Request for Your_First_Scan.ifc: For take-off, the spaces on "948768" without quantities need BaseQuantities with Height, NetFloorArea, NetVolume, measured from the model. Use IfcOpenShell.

First a look at what the model holds.

```python
import ifcopenshell
import ifcopenshell.util.element
import ifcopenshell.util.unit

model = ifcopenshell.open("Your_First_Scan.ifc")
print(model.schema)
for unit_type in ("LENGTHUNIT", "AREAUNIT", "VOLUMEUNIT"):
    print(unit_type, ifcopenshell.util.unit.calculate_unit_scale(model, unit_type))
storey = next(s for s in model.by_type("IfcBuildingStorey") if s.Name == "948768")
spaces = [e for e in ifcopenshell.util.element.get_decomposition(storey) if e.is_a("IfcSpace")]
for e in sorted(spaces, key=lambda e: e.id()):
    print(e.id(), e.is_a(), e.Name, list(ifcopenshell.util.element.get_psets(e, qtos_only=True)), sep=" | ")
```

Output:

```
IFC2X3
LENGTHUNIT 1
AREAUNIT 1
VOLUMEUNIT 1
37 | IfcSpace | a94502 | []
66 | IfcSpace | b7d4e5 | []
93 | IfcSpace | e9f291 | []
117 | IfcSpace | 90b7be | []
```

```python
import ifcopenshell
import ifcopenshell.api.pset
import ifcopenshell.geom
import ifcopenshell.util.element
import ifcopenshell.util.shape
import ifcopenshell.util.unit

model = ifcopenshell.open("Your_First_Scan.ifc")
unit_scale = ifcopenshell.util.unit.calculate_unit_scale(model)
area_scale = ifcopenshell.util.unit.calculate_unit_scale(model, "AREAUNIT")
volume_scale = ifcopenshell.util.unit.calculate_unit_scale(model, "VOLUMEUNIT")
settings = ifcopenshell.geom.settings()

storey = next(s for s in model.by_type("IfcBuildingStorey") if s.Name == "948768")
spaces = [e for e in ifcopenshell.util.element.get_decomposition(storey) if e.is_a("IfcSpace")]

for e in sorted(spaces, key=lambda e: e.id()):
    if ifcopenshell.util.element.get_psets(e, qtos_only=True, should_inherit=False):
        continue
    # Geometry comes back in metres, in the element's own axes.
    shape = ifcopenshell.geom.create_shape(settings, e)
    values = {
        "Height": ifcopenshell.util.shape.get_z(shape.geometry) / unit_scale,
        "NetFloorArea": ifcopenshell.util.shape.get_footprint_area(shape.geometry) / area_scale,
        "NetVolume": ifcopenshell.util.shape.get_volume(shape.geometry) / volume_scale,
    }
    qto = ifcopenshell.api.pset.add_qto(model, product=e, name="BaseQuantities")
    ifcopenshell.api.pset.edit_qto(model, qto=qto, properties=values)
    print(e.id(), {k: round(v, 3) for k, v in values.items()})

model.write("Your_First_Scan_updated.ifc")
```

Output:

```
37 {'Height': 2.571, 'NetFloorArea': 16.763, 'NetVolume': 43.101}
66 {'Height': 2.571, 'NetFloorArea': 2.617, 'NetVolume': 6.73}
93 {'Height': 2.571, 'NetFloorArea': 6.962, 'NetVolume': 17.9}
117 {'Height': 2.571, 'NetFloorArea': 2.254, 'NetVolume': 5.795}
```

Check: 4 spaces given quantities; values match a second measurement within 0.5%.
